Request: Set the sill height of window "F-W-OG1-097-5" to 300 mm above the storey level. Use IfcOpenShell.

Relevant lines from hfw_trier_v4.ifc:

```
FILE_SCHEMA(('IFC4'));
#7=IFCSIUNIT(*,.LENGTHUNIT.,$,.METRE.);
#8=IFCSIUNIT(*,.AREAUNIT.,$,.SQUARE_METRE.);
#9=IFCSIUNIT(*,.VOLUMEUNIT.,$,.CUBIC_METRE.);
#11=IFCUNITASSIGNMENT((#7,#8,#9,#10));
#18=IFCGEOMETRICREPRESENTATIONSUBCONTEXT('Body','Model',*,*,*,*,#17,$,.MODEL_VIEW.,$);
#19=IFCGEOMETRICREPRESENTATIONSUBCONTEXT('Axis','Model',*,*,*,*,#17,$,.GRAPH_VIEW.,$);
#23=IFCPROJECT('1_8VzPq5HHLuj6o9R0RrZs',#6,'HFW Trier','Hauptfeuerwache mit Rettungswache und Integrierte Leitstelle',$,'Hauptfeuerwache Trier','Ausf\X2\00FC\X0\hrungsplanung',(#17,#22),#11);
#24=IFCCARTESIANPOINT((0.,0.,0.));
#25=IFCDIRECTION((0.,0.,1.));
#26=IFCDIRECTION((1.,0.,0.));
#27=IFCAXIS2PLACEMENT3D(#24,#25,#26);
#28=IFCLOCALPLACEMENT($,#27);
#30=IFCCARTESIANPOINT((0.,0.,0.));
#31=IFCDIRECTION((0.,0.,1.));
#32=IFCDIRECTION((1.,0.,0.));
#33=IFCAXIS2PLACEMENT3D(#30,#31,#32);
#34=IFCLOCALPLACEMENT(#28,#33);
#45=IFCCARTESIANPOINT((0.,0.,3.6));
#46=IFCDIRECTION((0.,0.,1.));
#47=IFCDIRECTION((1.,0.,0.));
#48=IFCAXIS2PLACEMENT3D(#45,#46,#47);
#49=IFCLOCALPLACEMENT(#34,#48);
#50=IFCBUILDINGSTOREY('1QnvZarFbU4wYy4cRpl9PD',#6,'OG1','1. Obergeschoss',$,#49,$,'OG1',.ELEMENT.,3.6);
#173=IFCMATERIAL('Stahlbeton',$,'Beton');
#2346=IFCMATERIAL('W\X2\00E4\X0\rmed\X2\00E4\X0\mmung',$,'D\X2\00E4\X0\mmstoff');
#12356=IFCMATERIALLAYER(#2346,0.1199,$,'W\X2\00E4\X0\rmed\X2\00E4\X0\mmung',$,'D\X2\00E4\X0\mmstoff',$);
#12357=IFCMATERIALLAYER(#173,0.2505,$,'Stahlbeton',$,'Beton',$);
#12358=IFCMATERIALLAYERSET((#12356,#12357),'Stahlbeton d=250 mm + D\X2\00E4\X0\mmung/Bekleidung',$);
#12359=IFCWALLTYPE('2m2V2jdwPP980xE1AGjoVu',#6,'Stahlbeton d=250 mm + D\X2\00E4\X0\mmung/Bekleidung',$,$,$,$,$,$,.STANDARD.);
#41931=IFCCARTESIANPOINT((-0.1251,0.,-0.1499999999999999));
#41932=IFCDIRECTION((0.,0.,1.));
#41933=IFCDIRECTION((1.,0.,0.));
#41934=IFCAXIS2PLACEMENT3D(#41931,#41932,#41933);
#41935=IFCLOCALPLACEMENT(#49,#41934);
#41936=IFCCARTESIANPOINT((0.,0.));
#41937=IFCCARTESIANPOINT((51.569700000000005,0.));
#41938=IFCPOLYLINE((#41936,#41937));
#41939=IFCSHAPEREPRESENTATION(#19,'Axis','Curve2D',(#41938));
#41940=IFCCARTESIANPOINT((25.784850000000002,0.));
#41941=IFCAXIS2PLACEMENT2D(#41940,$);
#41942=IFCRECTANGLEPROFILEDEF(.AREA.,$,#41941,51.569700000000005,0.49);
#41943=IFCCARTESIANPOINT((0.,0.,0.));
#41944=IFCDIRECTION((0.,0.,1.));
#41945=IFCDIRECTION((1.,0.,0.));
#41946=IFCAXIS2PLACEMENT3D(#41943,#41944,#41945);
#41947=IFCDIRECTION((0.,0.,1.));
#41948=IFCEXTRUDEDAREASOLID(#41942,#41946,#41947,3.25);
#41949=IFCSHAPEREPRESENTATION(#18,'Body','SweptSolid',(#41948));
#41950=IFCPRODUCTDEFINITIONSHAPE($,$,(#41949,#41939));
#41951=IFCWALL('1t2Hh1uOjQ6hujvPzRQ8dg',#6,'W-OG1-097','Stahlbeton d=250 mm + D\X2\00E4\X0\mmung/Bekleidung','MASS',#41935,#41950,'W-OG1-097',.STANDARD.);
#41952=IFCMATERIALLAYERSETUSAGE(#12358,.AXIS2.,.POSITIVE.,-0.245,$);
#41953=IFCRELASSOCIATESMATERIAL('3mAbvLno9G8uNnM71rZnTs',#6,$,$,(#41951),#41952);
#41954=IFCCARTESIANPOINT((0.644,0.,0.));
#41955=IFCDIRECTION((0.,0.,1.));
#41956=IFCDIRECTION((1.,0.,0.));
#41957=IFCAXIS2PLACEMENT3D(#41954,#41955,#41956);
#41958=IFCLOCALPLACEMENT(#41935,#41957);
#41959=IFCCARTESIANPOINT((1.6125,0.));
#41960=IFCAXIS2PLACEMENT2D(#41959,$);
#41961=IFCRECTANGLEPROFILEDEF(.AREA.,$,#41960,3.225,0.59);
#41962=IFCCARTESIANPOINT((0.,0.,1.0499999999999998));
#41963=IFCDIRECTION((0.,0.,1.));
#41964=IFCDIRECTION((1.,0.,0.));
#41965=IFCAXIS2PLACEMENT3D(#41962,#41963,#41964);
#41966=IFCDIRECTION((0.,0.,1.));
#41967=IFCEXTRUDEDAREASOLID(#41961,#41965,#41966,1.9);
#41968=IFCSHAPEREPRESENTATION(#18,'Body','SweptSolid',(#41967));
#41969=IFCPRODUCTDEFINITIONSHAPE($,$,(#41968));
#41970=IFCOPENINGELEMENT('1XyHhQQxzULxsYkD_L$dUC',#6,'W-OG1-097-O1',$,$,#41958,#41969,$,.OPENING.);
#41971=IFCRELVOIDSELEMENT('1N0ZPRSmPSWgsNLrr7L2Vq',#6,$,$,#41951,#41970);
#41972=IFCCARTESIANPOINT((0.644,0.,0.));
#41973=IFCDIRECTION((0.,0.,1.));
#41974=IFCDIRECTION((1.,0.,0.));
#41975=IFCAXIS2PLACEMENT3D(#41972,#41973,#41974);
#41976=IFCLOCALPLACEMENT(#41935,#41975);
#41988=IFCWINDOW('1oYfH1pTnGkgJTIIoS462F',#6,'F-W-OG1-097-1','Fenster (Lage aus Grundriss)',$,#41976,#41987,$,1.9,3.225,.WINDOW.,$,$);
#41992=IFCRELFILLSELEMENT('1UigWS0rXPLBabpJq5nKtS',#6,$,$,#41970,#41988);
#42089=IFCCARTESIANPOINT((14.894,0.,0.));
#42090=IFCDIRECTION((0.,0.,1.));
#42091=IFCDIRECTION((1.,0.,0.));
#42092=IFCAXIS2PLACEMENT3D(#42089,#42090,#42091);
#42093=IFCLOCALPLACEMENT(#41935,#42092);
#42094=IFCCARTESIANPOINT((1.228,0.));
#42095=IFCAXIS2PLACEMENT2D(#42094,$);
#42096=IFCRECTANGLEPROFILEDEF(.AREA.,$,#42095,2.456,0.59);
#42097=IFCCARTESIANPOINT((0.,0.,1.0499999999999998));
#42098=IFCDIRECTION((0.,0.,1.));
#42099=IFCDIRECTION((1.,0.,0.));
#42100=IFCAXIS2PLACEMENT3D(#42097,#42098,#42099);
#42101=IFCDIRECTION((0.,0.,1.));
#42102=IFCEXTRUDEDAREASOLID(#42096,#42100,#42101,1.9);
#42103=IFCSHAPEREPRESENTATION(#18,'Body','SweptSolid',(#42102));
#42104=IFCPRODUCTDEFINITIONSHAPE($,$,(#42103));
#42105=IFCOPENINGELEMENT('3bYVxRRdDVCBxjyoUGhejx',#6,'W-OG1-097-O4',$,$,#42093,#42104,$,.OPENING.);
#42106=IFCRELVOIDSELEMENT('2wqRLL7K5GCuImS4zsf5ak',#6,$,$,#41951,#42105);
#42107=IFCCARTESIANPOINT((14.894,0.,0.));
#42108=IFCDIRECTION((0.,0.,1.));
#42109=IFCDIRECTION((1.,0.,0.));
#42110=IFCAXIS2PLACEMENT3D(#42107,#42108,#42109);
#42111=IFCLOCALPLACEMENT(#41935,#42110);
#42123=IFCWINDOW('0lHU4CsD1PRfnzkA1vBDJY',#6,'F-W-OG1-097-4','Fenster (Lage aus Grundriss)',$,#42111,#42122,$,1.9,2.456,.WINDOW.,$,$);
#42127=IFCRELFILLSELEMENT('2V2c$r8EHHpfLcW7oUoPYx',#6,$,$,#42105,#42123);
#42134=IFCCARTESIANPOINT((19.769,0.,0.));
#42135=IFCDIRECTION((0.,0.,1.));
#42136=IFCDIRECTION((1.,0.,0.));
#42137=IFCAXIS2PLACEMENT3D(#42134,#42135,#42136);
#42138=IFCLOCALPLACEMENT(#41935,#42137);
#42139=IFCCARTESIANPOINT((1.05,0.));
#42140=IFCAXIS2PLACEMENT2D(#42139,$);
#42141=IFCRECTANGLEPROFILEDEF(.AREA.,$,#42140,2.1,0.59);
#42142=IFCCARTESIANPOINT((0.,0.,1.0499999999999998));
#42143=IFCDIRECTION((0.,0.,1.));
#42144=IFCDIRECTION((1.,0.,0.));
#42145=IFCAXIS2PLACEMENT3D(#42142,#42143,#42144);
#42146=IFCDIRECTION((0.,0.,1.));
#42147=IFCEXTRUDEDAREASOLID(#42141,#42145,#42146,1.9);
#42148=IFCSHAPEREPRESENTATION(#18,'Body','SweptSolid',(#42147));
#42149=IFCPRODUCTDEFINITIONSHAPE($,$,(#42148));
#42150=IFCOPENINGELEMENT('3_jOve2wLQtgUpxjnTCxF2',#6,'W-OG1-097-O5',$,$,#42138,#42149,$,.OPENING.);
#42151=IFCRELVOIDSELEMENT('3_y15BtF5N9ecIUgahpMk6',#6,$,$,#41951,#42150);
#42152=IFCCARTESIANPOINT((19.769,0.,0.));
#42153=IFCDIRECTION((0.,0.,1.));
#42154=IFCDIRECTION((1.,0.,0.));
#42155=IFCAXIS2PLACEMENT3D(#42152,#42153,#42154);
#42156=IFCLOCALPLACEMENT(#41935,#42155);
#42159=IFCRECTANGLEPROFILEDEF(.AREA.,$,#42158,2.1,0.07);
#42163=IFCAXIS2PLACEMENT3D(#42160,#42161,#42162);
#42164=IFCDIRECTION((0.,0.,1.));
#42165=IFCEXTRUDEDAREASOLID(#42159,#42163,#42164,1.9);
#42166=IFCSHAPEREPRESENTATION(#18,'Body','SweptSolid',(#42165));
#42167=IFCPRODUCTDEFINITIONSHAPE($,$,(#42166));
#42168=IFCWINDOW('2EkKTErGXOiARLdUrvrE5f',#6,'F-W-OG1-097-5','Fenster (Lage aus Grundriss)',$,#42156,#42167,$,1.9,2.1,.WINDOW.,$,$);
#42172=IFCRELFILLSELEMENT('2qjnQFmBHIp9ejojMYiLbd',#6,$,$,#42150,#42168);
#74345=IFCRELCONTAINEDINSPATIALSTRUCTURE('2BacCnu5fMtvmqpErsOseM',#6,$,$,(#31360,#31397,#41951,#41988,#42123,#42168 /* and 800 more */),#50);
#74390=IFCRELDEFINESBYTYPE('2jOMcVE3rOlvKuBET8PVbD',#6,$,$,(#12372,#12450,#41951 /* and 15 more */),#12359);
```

```python
import numpy as np
import ifcopenshell
import ifcopenshell.api.geometry
import ifcopenshell.geom
import ifcopenshell.util.element
import ifcopenshell.util.placement
import ifcopenshell.util.shape
import ifcopenshell.util.unit

model = ifcopenshell.open("hfw_trier_v4.ifc")
unit_scale = ifcopenshell.util.unit.calculate_unit_scale(model)

window = model.by_id(42168)
opening = window.FillsVoids[0].RelatingOpeningElement
storey = ifcopenshell.util.element.get_container(window, ifc_class="IfcBuildingStorey")
level = ifcopenshell.util.placement.get_local_placement(storey.ObjectPlacement)[2, 3]

# The opening's origin need not be at the sill, so measure its lowest point.
shape = ifcopenshell.geom.create_shape(ifcopenshell.geom.settings(), opening)
bottom = ifcopenshell.util.shape.get_shape_bottom_elevation(shape, shape.geometry) / unit_scale
dz = level + 0.3 / unit_scale - bottom

shift = np.array([0.0, 0.0, dz])
# The window is not placed relative to its opening, so move both.
for product in (opening, window):
    matrix = ifcopenshell.util.placement.get_local_placement(product.ObjectPlacement)
    matrix[:3, 3] += shift
    ifcopenshell.api.geometry.edit_object_placement(model, product=product, matrix=matrix, is_si=False)

print(f"moved by {dz * unit_scale:+.3f} m")

model.write("hfw_trier_v4_updated.ifc")
```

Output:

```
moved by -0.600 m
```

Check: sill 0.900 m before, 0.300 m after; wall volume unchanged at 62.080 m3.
